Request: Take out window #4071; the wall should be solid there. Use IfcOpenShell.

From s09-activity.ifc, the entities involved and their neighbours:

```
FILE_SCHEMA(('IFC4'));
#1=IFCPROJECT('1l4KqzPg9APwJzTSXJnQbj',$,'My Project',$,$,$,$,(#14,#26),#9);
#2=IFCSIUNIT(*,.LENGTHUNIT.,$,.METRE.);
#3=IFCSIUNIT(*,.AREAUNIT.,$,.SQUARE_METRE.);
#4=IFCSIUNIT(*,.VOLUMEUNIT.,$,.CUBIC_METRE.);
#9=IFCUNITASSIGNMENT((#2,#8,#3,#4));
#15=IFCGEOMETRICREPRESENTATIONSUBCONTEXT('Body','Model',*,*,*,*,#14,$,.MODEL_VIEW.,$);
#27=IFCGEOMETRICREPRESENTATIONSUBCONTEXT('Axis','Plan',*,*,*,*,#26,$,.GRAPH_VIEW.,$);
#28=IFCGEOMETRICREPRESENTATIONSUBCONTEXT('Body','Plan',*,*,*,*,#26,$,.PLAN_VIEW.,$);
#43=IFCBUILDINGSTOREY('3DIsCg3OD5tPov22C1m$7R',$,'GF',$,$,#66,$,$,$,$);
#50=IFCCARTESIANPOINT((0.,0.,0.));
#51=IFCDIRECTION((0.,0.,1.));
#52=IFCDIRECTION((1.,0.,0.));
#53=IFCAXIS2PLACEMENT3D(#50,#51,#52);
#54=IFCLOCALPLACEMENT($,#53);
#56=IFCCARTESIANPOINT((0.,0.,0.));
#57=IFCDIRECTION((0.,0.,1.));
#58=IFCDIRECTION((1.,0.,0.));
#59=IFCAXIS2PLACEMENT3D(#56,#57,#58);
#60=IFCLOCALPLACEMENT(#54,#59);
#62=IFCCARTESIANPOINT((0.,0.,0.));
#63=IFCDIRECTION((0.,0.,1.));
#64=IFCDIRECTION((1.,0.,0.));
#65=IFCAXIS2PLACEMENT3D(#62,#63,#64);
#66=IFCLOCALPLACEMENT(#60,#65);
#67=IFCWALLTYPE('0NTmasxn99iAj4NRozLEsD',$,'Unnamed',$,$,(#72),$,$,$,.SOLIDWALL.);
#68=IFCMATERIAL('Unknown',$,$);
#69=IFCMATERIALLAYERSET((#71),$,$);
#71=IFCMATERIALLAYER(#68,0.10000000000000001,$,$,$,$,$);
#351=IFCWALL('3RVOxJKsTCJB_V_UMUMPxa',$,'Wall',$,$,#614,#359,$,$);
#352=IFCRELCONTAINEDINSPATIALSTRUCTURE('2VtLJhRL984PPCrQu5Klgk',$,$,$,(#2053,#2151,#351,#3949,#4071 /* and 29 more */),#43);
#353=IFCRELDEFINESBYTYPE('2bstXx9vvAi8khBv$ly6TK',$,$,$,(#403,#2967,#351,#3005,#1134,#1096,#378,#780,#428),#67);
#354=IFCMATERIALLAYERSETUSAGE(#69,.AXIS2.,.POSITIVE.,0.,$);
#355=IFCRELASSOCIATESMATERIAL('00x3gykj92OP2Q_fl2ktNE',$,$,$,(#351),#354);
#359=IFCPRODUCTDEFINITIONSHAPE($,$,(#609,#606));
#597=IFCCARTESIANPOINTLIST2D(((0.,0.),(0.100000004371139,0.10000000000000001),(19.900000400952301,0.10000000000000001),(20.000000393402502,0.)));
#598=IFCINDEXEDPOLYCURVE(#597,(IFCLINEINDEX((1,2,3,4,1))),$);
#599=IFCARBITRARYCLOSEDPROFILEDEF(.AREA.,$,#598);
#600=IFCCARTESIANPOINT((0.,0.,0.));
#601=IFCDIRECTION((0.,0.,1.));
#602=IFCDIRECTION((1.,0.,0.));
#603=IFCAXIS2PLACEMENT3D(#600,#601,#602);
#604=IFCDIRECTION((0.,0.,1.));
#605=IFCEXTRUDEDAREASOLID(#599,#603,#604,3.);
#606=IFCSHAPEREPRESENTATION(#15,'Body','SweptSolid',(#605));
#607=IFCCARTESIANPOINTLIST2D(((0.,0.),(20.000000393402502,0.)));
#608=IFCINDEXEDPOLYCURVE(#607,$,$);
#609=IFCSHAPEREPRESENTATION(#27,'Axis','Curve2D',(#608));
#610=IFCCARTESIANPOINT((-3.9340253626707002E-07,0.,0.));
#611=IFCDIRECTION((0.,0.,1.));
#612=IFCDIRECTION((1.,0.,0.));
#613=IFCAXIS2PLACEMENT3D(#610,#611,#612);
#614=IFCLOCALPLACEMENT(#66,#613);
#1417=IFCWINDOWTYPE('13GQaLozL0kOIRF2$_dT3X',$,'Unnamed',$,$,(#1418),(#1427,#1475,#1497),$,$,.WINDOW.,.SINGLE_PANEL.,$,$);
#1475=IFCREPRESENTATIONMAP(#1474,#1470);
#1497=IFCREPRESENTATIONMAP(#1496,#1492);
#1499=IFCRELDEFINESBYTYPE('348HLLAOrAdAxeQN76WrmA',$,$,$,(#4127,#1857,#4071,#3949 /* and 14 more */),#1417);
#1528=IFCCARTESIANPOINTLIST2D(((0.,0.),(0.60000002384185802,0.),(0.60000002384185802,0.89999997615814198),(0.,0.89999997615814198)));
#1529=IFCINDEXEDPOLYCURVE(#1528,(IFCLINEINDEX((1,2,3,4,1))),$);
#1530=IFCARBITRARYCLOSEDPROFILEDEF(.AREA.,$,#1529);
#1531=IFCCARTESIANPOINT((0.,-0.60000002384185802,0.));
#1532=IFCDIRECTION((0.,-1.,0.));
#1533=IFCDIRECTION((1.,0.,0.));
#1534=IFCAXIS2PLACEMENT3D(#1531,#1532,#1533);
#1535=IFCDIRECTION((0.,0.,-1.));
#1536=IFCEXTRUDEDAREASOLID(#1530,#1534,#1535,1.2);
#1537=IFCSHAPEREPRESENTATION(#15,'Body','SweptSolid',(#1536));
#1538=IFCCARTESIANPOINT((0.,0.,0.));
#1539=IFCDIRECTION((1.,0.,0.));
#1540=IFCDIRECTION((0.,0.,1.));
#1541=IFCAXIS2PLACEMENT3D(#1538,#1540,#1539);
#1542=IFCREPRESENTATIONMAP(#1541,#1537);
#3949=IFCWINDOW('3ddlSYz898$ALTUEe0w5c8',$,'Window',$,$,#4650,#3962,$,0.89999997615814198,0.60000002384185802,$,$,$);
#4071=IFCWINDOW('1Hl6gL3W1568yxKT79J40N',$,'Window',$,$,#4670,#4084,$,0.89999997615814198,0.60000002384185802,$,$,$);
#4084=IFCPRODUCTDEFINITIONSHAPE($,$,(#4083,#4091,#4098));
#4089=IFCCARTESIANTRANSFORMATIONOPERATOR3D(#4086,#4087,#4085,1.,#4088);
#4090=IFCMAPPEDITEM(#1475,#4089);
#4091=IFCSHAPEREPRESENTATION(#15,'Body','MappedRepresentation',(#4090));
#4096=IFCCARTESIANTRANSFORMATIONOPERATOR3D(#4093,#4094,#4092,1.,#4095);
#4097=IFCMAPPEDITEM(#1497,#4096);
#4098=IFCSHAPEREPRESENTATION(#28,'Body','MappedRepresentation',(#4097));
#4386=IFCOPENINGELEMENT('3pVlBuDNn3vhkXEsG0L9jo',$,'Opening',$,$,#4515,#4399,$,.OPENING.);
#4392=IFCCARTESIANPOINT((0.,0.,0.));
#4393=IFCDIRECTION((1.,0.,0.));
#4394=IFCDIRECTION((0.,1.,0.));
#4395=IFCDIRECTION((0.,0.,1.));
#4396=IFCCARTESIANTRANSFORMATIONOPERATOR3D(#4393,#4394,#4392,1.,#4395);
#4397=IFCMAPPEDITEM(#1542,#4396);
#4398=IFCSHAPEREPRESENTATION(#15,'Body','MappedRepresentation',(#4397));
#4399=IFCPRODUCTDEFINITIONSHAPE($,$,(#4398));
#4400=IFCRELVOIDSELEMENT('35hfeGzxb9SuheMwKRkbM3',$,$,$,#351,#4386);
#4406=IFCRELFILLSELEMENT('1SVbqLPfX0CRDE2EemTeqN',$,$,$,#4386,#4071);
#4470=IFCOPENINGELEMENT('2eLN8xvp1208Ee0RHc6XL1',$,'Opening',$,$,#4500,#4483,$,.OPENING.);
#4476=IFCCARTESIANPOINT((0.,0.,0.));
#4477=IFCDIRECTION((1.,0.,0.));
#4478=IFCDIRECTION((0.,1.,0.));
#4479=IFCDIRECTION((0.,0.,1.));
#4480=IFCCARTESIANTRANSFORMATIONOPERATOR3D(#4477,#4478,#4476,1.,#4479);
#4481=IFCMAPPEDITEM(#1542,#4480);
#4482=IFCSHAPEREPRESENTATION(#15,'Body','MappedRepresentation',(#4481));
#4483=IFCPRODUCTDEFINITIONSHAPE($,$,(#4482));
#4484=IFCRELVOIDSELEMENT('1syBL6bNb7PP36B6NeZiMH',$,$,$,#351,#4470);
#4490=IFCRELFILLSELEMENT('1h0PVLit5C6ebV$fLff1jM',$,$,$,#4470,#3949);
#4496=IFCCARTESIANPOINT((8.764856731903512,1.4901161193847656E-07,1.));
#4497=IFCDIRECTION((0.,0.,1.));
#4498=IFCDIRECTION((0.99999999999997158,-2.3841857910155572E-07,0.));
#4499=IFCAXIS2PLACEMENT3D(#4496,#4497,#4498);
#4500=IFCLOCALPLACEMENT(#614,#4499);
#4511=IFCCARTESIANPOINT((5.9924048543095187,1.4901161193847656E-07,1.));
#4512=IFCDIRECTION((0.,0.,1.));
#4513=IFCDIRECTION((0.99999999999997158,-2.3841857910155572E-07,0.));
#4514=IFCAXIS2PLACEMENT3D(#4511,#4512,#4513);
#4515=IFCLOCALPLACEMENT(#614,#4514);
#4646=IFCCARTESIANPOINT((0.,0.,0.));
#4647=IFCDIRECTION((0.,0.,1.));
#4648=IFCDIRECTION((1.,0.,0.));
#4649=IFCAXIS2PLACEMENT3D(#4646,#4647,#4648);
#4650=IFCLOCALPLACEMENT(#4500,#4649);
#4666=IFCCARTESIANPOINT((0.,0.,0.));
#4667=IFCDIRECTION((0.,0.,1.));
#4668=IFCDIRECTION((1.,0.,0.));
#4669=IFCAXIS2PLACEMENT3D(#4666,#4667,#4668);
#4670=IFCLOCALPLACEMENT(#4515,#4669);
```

```python
import ifcopenshell
import ifcopenshell.api.feature
import ifcopenshell.api.root
import ifcopenshell.geom
import ifcopenshell.util.shape

model = ifcopenshell.open("s09-activity.ifc")
settings = ifcopenshell.geom.settings()


def volume(element):
    """Net volume in cubic metres, openings subtracted."""
    shape = ifcopenshell.geom.create_shape(settings, element)
    return ifcopenshell.util.shape.get_volume(shape.geometry)


window = model.by_guid("1Hl6gL3W1568yxKT79J40N")
opening = window.FillsVoids[0].RelatingOpeningElement
wall = opening.VoidsElements[0].RelatingBuildingElement
before = volume(wall)

ifcopenshell.api.root.remove_product(model, product=window)
ifcopenshell.api.feature.remove_feature(model, feature=opening)

after = volume(wall)

print(f"wall volume {before:.3f} -> {after:.3f} m3")

model.write("s09-activity-out.ifc")
```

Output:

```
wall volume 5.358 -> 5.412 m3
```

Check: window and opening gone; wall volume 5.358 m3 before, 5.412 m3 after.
